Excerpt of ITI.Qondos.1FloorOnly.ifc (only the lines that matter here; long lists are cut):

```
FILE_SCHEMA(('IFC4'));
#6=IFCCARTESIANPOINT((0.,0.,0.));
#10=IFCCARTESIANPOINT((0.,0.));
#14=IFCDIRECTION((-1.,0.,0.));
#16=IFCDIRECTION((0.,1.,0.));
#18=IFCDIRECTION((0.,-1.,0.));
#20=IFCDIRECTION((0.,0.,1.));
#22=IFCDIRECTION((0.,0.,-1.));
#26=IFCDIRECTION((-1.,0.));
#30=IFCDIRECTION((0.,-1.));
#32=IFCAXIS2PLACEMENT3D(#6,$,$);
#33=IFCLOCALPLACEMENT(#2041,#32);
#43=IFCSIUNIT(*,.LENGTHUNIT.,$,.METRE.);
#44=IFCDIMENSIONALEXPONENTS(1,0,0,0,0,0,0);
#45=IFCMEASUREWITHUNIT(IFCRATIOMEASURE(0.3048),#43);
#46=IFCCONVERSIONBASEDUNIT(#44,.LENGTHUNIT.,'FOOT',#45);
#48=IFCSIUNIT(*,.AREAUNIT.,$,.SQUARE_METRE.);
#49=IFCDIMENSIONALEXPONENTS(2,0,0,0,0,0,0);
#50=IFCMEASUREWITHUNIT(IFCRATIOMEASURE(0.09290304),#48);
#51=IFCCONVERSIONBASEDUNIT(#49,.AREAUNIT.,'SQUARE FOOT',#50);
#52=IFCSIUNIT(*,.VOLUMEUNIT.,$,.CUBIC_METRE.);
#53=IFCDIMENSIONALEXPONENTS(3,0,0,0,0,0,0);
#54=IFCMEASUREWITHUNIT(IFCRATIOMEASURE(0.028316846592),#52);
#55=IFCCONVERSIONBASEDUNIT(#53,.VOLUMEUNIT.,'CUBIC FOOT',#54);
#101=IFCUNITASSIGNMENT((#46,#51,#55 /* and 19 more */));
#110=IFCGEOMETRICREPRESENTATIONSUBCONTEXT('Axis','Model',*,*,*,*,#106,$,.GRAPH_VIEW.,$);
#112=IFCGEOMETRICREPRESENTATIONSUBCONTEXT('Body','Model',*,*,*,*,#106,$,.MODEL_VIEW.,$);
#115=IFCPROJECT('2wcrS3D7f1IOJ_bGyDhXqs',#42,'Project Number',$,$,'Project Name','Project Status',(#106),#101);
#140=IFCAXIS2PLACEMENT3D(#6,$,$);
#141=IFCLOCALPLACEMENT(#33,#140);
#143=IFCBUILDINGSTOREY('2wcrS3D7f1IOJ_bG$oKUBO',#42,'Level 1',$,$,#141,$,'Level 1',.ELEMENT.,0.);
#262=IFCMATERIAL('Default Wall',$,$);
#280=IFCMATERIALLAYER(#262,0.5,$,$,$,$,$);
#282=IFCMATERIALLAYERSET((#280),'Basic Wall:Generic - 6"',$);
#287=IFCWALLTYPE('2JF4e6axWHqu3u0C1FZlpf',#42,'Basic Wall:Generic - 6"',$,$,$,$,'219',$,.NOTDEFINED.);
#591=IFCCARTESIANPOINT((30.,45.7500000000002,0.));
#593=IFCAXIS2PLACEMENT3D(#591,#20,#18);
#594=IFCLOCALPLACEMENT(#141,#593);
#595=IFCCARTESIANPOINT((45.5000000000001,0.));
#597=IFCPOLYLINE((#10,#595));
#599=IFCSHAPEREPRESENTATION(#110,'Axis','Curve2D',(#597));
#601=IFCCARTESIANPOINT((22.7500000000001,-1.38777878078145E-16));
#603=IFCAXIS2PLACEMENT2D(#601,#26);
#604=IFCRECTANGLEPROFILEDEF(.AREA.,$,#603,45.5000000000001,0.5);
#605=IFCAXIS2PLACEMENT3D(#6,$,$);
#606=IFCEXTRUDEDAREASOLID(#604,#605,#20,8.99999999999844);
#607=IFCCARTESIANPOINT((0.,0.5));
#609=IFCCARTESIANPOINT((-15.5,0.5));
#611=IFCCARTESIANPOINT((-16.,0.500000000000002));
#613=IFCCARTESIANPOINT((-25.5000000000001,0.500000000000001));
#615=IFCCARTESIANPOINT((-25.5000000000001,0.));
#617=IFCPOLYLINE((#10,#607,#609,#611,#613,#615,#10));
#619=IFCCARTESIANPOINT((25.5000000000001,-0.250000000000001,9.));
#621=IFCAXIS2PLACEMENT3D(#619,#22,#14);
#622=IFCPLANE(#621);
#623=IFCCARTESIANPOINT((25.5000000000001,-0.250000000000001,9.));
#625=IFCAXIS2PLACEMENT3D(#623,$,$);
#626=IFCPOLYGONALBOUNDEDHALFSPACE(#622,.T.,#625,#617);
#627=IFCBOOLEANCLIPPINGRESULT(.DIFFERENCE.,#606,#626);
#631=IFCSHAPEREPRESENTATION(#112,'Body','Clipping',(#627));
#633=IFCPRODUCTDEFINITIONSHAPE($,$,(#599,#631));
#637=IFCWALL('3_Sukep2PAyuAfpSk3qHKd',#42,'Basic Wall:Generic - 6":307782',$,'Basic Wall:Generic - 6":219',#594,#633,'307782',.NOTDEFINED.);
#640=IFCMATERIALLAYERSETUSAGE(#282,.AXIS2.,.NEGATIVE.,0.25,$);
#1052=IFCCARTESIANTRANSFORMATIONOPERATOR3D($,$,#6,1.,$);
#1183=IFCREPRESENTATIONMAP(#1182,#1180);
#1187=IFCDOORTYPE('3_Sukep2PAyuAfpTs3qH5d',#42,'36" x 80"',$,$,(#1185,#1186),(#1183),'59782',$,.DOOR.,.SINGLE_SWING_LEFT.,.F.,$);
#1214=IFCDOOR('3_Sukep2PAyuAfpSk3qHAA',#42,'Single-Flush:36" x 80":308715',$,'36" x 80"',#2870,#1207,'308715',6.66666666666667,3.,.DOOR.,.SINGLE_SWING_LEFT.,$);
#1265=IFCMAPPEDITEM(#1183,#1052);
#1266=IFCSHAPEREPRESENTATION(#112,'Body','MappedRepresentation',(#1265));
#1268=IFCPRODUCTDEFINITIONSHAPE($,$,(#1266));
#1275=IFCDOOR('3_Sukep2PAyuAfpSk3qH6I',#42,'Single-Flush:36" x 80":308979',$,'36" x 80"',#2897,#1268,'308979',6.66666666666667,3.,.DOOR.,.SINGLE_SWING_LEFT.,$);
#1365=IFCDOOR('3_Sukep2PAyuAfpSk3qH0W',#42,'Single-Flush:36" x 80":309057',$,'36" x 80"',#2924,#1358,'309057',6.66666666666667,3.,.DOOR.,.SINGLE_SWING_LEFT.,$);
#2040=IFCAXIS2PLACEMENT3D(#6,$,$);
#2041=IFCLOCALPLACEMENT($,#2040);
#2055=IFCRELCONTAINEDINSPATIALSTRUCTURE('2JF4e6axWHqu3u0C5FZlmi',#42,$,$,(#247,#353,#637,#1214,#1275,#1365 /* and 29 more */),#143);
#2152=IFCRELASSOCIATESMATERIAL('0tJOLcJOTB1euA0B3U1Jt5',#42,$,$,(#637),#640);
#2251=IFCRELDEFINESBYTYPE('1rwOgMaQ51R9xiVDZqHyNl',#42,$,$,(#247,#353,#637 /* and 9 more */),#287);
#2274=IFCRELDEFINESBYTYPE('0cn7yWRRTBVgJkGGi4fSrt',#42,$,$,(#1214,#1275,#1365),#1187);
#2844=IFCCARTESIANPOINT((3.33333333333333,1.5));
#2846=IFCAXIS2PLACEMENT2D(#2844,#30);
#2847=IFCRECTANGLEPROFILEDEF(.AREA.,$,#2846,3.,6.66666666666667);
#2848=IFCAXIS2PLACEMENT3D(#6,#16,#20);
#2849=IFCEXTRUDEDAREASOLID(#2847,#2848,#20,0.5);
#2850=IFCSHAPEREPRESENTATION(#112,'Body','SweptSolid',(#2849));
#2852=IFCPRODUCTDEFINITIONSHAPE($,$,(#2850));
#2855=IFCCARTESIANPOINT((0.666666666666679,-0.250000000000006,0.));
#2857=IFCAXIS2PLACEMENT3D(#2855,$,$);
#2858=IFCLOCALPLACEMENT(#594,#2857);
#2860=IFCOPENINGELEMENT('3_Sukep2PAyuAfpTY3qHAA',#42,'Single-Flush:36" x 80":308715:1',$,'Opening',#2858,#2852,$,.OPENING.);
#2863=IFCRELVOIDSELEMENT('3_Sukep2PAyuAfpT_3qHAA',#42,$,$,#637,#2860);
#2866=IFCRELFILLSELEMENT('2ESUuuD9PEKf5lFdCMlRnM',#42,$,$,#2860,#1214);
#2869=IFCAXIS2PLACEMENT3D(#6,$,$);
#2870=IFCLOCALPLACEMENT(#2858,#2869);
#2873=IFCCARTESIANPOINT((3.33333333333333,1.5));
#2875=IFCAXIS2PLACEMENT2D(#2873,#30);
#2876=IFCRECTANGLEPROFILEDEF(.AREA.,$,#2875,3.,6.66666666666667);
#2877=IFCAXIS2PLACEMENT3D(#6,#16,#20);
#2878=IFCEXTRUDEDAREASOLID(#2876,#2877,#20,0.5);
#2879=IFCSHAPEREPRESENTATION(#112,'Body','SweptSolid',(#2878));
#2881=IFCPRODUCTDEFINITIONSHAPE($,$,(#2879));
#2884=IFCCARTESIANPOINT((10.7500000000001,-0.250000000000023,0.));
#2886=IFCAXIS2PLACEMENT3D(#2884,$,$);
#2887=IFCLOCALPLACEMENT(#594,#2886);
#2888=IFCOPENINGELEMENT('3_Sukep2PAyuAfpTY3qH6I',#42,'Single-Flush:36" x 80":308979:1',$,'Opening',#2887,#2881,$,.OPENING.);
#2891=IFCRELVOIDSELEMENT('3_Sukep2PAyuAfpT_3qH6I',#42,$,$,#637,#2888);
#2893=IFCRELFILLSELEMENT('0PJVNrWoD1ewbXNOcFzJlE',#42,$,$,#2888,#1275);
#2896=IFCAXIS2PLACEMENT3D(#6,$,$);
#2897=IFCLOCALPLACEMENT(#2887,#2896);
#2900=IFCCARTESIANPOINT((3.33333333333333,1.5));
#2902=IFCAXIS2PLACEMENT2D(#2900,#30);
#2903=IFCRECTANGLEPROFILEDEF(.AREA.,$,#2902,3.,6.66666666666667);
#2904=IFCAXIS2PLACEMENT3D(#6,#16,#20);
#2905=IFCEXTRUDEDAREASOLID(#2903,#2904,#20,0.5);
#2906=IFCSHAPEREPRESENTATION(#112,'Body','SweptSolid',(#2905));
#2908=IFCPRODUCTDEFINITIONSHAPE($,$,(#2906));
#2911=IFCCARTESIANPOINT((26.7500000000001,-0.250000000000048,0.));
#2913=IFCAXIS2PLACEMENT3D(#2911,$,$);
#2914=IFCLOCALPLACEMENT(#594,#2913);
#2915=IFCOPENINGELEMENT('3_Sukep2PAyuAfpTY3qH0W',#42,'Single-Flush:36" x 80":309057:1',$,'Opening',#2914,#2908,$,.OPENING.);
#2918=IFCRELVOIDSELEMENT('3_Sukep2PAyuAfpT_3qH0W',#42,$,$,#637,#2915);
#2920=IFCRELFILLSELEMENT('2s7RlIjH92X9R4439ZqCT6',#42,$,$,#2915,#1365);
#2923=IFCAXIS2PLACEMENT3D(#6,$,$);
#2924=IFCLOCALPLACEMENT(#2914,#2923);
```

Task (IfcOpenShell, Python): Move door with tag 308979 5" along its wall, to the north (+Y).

```python
import ifcopenshell
import ifcopenshell.api.geometry
import ifcopenshell.util.placement
import ifcopenshell.util.unit

model = ifcopenshell.open("ITI.Qondos.1FloorOnly.ifc")
unit_scale = ifcopenshell.util.unit.calculate_unit_scale(model)

door = model.by_guid("3_Sukep2PAyuAfpSk3qH6I")
opening = door.FillsVoids[0].RelatingOpeningElement
wall = opening.VoidsElements[0].RelatingBuildingElement

wall_matrix = ifcopenshell.util.placement.get_local_placement(wall.ObjectPlacement)
shift = wall_matrix[:3, 0] * -5 * 0.0254 / unit_scale
before = ifcopenshell.util.placement.get_local_placement(door.ObjectPlacement)[:3, 3].copy()

# The door is placed relative to its opening, so it follows when the opening moves.
matrix = ifcopenshell.util.placement.get_local_placement(opening.ObjectPlacement)
matrix[:3, 3] += shift
ifcopenshell.api.geometry.edit_object_placement(
    model, product=opening, matrix=matrix, is_si=False, should_transform_children=True
)

after = ifcopenshell.util.placement.get_local_placement(door.ObjectPlacement)[:3, 3]
print("door moved by", (after - before).round(3) + 0.0)

model.write("ITI.Qondos.1FloorOnly_updated.ifc")
```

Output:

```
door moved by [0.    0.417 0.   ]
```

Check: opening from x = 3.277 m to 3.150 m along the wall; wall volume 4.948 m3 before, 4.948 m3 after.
